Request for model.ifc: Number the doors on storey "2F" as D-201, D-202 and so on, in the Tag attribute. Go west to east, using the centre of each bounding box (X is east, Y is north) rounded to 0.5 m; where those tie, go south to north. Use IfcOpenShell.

First a look at what the model holds.

```python
import ifcopenshell
import ifcopenshell.util.element
import ifcopenshell.util.placement

model = ifcopenshell.open("model.ifc")
print(model.schema)
storey = next(s for s in model.by_type("IfcBuildingStorey") if s.Name == "2F")
doors = [e for e in ifcopenshell.util.element.get_decomposition(storey) if e.is_a("IfcDoor")]
for e in sorted(doors, key=lambda e: e.id()):
    origin = ifcopenshell.util.placement.get_local_placement(e.ObjectPlacement)[:3, 3]
    print(e.id(), e.Tag, e.Name, origin.round(2) + 0.0, sep=" | ")
```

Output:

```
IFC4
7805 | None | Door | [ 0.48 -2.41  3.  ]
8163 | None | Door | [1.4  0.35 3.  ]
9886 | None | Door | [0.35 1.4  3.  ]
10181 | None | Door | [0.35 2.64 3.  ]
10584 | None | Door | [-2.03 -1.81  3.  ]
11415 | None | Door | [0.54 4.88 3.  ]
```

```python
import ifcopenshell
import ifcopenshell.geom
import ifcopenshell.util.element
import ifcopenshell.util.shape

model = ifcopenshell.open("model.ifc")
settings = ifcopenshell.geom.settings()
settings.set("use-world-coords", True)


def centre(element):
    shape = ifcopenshell.geom.create_shape(settings, element)
    return ifcopenshell.util.shape.get_bbox_centroid(shape.geometry)


storey = next(s for s in model.by_type("IfcBuildingStorey") if s.Name == "2F")
doors = [e for e in ifcopenshell.util.element.get_decomposition(storey) if e.is_a("IfcDoor")]

# Insertion points can sit at a corner or the storey origin, so sort by the geometry (in metres).
centres = {e: centre(e) for e in doors}
doors.sort(key=lambda e: (round(centres[e][0] / 0.5), centres[e][1]))

for i, e in enumerate(doors, start=1):
    number = f"D-2{i:02d}"
    e.Tag = number
    print(e.id(), number)

model.write("model_v2.ifc")
```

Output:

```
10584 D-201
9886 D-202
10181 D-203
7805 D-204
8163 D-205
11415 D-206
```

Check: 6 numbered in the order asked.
